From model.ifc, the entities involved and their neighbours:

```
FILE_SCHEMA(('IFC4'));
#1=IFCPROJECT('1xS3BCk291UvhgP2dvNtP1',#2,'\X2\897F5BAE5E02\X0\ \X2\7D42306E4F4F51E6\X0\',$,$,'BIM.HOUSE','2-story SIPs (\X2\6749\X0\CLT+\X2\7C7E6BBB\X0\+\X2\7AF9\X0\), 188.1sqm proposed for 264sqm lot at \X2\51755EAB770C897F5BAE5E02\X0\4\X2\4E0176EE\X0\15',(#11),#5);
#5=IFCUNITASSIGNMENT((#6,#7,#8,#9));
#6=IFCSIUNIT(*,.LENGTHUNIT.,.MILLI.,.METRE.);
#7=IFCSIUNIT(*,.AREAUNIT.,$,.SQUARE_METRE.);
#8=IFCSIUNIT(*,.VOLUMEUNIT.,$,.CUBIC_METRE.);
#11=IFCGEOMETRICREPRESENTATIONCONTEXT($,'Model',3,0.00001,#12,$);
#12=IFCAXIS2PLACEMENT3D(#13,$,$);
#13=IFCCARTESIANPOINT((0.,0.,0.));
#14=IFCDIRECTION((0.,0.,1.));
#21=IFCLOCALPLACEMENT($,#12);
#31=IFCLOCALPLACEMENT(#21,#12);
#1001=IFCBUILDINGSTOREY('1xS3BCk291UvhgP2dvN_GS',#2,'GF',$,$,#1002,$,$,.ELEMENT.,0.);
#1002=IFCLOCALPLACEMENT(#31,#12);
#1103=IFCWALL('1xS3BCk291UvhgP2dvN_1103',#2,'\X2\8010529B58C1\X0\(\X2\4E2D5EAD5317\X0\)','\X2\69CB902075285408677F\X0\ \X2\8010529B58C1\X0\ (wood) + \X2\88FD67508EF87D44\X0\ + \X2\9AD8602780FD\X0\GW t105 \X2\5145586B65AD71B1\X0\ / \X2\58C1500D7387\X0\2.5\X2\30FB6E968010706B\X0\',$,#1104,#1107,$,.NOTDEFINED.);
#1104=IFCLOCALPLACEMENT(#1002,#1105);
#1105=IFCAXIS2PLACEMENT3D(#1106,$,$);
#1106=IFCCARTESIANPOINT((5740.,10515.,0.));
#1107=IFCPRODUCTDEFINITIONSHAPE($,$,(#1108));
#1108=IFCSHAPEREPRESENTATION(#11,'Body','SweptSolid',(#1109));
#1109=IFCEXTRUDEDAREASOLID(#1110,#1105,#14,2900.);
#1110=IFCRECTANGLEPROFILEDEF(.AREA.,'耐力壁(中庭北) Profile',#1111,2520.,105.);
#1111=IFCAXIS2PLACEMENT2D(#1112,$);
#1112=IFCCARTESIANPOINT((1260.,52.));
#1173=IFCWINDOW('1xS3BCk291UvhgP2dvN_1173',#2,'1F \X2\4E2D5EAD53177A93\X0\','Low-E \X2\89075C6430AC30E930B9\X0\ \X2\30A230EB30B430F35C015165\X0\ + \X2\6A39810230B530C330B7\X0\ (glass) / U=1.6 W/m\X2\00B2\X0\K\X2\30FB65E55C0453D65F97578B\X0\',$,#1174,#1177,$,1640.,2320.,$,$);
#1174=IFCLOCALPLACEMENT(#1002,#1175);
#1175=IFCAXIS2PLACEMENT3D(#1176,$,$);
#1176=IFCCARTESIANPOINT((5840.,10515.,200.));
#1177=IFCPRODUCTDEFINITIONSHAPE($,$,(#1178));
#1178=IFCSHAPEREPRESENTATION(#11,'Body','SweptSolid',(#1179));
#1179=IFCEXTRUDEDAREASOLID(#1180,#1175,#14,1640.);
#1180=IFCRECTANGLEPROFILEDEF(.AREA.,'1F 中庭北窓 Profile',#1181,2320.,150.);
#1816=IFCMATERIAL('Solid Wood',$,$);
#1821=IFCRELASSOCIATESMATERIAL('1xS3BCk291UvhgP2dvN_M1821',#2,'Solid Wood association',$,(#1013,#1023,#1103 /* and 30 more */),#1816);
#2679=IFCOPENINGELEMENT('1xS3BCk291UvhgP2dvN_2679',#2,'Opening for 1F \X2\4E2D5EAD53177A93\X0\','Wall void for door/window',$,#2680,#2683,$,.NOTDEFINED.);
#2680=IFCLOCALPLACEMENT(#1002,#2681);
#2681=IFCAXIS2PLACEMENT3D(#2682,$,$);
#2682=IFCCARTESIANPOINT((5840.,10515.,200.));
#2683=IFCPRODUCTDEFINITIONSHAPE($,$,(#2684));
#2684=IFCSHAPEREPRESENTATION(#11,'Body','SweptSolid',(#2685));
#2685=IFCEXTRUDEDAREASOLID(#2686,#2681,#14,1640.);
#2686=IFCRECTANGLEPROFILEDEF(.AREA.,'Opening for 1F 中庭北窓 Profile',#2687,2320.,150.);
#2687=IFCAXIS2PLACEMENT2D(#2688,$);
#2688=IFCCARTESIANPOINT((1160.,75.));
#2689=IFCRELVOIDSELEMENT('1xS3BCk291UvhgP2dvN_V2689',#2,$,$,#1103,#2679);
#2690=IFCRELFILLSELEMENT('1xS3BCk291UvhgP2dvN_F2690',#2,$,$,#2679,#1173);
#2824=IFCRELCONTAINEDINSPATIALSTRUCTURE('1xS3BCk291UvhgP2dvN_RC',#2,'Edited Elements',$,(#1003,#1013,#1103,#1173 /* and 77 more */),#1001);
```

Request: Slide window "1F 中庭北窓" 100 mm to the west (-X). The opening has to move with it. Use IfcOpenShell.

```python
import ifcopenshell
import ifcopenshell.api.geometry
import ifcopenshell.util.placement
import ifcopenshell.util.unit

model = ifcopenshell.open("model.ifc")
unit_scale = ifcopenshell.util.unit.calculate_unit_scale(model)

window = model.by_id(1173)
opening = window.FillsVoids[0].RelatingOpeningElement
wall = opening.VoidsElements[0].RelatingBuildingElement

wall_matrix = ifcopenshell.util.placement.get_local_placement(wall.ObjectPlacement)
shift = wall_matrix[:3, 0] * -0.1 / unit_scale
before = ifcopenshell.util.placement.get_local_placement(window.ObjectPlacement)[:3, 3].copy()

# The window is not placed relative to its opening, so move both.
for product in (opening, window):
    matrix = ifcopenshell.util.placement.get_local_placement(product.ObjectPlacement)
    matrix[:3, 3] += shift
    ifcopenshell.api.geometry.edit_object_placement(model, product=product, matrix=matrix, is_si=False)

after = ifcopenshell.util.placement.get_local_placement(window.ObjectPlacement)[:3, 3]
print("window moved by", (after - before).round(3) + 0.0)

model.write("model_rev.ifc")
```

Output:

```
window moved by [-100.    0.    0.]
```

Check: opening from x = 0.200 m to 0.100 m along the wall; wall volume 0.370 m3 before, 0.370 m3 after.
